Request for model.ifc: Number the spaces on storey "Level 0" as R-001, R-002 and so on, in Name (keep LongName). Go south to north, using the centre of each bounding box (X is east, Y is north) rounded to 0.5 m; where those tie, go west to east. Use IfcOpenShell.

First a look at what the model holds.

```python
import ifcopenshell
import ifcopenshell.util.element
import ifcopenshell.util.placement

model = ifcopenshell.open("model.ifc")
print(model.schema)
storey = next(s for s in model.by_type("IfcBuildingStorey") if s.Name == "Level 0")
spaces = [e for e in ifcopenshell.util.element.get_decomposition(storey) if e.is_a("IfcSpace")]
for e in sorted(spaces, key=lambda e: e.id()):
    origin = ifcopenshell.util.placement.get_local_placement(e.ObjectPlacement)[:3, 3]
    print(e.id(), e.Name, e.LongName, origin.round(2) + 0.0, sep=" | ")
```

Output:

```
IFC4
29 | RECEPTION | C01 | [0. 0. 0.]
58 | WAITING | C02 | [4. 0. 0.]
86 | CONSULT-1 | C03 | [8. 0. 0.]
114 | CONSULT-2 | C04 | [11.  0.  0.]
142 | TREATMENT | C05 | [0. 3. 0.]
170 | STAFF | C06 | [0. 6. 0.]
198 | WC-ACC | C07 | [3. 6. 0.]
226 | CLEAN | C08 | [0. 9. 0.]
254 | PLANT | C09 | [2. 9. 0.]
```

```python
import ifcopenshell
import ifcopenshell.geom
import ifcopenshell.util.element
import ifcopenshell.util.shape

model = ifcopenshell.open("model.ifc")
settings = ifcopenshell.geom.settings()
settings.set("use-world-coords", True)


def centre(element):
    shape = ifcopenshell.geom.create_shape(settings, element)
    return ifcopenshell.util.shape.get_bbox_centroid(shape.geometry)


storey = next(s for s in model.by_type("IfcBuildingStorey") if s.Name == "Level 0")
spaces = [e for e in ifcopenshell.util.element.get_decomposition(storey) if e.is_a("IfcSpace")]

# Insertion points can sit at a corner or the storey origin, so sort by the geometry (in metres).
centres = {e: centre(e) for e in spaces}
spaces.sort(key=lambda e: (round(centres[e][1] / 0.5), centres[e][0]))

for i, e in enumerate(spaces, start=1):
    number = f"R-0{i:02d}"
    e.Name = number
    print(e.id(), number)

model.write("model_edited.ifc")
```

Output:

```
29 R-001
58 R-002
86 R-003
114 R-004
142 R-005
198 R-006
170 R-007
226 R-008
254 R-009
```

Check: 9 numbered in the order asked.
